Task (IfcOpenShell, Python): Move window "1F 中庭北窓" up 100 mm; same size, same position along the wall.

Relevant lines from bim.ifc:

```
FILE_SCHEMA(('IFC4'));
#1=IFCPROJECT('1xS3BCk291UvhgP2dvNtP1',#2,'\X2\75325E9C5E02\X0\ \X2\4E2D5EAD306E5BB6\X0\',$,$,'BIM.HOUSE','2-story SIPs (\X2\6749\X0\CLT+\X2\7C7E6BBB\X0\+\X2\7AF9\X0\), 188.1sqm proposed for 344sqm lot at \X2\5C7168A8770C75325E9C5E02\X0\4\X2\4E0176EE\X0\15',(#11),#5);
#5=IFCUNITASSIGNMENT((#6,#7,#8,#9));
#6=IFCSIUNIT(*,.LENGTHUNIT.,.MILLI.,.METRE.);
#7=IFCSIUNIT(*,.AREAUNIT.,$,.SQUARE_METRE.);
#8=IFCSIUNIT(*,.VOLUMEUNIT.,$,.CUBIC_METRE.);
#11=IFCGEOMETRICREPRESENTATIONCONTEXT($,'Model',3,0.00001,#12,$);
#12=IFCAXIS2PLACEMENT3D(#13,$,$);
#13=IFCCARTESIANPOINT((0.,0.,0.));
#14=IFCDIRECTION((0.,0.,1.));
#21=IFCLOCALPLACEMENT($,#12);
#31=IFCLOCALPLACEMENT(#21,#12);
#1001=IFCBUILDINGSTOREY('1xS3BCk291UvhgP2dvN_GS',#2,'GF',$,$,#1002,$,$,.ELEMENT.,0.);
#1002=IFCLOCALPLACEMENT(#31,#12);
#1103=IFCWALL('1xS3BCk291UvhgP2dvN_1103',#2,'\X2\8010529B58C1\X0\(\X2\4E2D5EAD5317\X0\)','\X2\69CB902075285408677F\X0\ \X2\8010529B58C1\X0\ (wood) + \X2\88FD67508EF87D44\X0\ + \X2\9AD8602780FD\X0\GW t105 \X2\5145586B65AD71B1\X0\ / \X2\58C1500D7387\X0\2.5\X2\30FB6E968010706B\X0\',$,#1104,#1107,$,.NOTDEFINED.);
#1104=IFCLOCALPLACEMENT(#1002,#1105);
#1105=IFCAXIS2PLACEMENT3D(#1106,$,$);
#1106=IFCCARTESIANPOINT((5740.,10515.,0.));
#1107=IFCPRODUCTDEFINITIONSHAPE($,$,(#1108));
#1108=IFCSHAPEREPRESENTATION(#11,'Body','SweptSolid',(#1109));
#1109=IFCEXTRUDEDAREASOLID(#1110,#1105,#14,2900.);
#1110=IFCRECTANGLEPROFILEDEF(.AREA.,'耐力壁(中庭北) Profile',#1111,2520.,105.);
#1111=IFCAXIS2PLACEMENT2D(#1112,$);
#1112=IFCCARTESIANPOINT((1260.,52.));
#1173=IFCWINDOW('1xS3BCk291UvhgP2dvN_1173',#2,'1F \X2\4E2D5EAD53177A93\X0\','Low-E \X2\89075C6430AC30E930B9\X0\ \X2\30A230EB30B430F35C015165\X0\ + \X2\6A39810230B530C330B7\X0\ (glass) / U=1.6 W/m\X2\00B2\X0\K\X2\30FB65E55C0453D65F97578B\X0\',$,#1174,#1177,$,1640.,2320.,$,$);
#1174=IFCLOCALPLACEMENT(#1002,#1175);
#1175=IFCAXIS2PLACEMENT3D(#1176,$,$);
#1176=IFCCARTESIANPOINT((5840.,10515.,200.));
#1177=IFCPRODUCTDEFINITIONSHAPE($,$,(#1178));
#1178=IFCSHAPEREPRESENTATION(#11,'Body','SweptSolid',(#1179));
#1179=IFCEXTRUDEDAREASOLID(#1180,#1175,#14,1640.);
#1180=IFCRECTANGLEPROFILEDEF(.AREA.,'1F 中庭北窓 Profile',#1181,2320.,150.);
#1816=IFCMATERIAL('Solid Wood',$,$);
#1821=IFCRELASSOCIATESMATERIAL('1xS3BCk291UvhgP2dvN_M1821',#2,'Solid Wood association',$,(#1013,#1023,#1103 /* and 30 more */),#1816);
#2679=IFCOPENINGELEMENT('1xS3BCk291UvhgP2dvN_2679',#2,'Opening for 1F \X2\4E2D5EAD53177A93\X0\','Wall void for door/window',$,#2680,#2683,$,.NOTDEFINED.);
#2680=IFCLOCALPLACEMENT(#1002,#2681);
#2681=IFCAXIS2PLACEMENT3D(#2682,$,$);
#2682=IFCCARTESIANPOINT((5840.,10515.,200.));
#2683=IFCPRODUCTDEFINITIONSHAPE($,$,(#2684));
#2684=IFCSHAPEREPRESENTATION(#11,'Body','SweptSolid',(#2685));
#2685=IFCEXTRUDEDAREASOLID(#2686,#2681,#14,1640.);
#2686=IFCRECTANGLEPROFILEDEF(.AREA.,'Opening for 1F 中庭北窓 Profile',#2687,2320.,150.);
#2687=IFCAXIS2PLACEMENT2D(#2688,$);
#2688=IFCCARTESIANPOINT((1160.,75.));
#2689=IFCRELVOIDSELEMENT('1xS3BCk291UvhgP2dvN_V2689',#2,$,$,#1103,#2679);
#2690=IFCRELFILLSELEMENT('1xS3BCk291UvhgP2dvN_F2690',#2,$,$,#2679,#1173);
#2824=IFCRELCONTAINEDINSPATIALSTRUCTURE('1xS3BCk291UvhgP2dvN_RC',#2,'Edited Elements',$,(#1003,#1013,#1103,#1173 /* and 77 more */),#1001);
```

```python
import numpy as np
import ifcopenshell
import ifcopenshell.api.geometry
import ifcopenshell.util.placement
import ifcopenshell.util.unit

model = ifcopenshell.open("bim.ifc")
unit_scale = ifcopenshell.util.unit.calculate_unit_scale(model)

window = model.by_guid("1xS3BCk291UvhgP2dvN_1173")
opening = window.FillsVoids[0].RelatingOpeningElement
dz = 100.0

shift = np.array([0.0, 0.0, dz])
# The window is not placed relative to its opening, so move both.
for product in (opening, window):
    matrix = ifcopenshell.util.placement.get_local_placement(product.ObjectPlacement)
    matrix[:3, 3] += shift
    ifcopenshell.api.geometry.edit_object_placement(model, product=product, matrix=matrix, is_si=False)

print(f"moved by {dz * unit_scale:+.3f} m")

model.write("bim_edited.ifc")
```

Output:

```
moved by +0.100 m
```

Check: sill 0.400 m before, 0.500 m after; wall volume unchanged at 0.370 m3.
